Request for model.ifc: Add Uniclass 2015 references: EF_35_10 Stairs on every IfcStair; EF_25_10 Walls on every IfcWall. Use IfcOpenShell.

First a look at what the model holds.

```python
import ifcopenshell

model = ifcopenshell.open("model.ifc")
print(model.schema)
print("classifications:", [c.Name for c in model.by_type("IfcClassification")])
for ifc_class in ("IfcDoor", "IfcRoof", "IfcStair", "IfcWall", "IfcWindow"):
    print(ifc_class, len(model.by_type(ifc_class)))
```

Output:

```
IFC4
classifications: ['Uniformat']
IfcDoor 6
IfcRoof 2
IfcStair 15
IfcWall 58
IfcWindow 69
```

```python
import ifcopenshell
import ifcopenshell.api.classification

model = ifcopenshell.open("model.ifc")

system = ifcopenshell.api.classification.add_classification(model, classification="Uniclass 2015")

codes = {
    "IfcStair": ("EF_35_10", "Stairs"),
    "IfcWall": ("EF_25_10", "Walls"),
}
for ifc_class, (code, name) in codes.items():
    products = model.by_type(ifc_class)
    ifcopenshell.api.classification.add_reference(
        model, products=products, classification=system, identification=code, name=name
    )
    print(code, len(products))

model.write("model_updated.ifc")
```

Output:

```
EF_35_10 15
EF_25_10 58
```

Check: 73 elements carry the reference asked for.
